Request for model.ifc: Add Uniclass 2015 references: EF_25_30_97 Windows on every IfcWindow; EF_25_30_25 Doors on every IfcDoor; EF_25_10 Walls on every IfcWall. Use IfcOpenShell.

First a look at what the model holds.

```python
import ifcopenshell

model = ifcopenshell.open("model.ifc")
print(model.schema)
print("classifications:", [c.Name for c in model.by_type("IfcClassification")])
for ifc_class in ("IfcDoor", "IfcRoof", "IfcStair", "IfcWall", "IfcWindow"):
    print(ifc_class, len(model.by_type(ifc_class)))
```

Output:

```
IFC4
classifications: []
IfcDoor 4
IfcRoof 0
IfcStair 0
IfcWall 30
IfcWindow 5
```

```python
import ifcopenshell
import ifcopenshell.api.classification

model = ifcopenshell.open("model.ifc")

system = ifcopenshell.api.classification.add_classification(model, classification="Uniclass 2015")

codes = {
    "IfcWindow": ("EF_25_30_97", "Windows"),
    "IfcDoor": ("EF_25_30_25", "Doors"),
    "IfcWall": ("EF_25_10", "Walls"),
}
for ifc_class, (code, name) in codes.items():
    products = model.by_type(ifc_class)
    ifcopenshell.api.classification.add_reference(
        model, products=products, classification=system, identification=code, name=name
    )
    print(code, len(products))

model.write("model_edited.ifc")
```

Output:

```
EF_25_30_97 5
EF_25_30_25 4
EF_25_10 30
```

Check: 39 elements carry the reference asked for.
